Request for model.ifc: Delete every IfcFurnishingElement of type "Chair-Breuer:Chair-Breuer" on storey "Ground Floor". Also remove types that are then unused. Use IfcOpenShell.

First a look at what the model holds.

```python
import ifcopenshell
import ifcopenshell.util.element

model = ifcopenshell.open("model.ifc")
print(model.schema)
storey = next(s for s in model.by_type("IfcBuildingStorey") if s.Name == "Ground Floor")
furniture = [e for e in ifcopenshell.util.element.get_decomposition(storey) if e.is_a("IfcFurnishingElement")]
seen = {}
for e in furniture:
    element_type = ifcopenshell.util.element.get_type(e)
    name = element_type.Name if element_type not in (None, e) else None
    seen[name] = seen.get(name, 0) + 1
for name, count in sorted(seen.items(), key=str):
    print(count, "x", name)
```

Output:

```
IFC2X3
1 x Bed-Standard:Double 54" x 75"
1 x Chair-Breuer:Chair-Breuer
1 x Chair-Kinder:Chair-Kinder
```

```python
import ifcopenshell
import ifcopenshell.api.root
import ifcopenshell.util.element

model = ifcopenshell.open("model.ifc")

storey = next(s for s in model.by_type("IfcBuildingStorey") if s.Name == "Ground Floor")
furniture = [e for e in ifcopenshell.util.element.get_decomposition(storey) if e.is_a("IfcFurnishingElement")]
targets = [e for e in furniture if (t := ifcopenshell.util.element.get_type(e)) not in (None, e) and t.Name == "Chair-Breuer:Chair-Breuer"]
types = {ifcopenshell.util.element.get_type(e) for e in targets} - {None, *targets}

for e in targets:
    ifcopenshell.api.root.remove_product(model, product=e)
print(len(targets), "removed")

unused = [t for t in types if not ifcopenshell.util.element.get_types(t)]
for t in unused:
    ifcopenshell.api.root.remove_product(model, product=t)
print(len(unused), "unused types removed")

model.write("model_edited.ifc")
```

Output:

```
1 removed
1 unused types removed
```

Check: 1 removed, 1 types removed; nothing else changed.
